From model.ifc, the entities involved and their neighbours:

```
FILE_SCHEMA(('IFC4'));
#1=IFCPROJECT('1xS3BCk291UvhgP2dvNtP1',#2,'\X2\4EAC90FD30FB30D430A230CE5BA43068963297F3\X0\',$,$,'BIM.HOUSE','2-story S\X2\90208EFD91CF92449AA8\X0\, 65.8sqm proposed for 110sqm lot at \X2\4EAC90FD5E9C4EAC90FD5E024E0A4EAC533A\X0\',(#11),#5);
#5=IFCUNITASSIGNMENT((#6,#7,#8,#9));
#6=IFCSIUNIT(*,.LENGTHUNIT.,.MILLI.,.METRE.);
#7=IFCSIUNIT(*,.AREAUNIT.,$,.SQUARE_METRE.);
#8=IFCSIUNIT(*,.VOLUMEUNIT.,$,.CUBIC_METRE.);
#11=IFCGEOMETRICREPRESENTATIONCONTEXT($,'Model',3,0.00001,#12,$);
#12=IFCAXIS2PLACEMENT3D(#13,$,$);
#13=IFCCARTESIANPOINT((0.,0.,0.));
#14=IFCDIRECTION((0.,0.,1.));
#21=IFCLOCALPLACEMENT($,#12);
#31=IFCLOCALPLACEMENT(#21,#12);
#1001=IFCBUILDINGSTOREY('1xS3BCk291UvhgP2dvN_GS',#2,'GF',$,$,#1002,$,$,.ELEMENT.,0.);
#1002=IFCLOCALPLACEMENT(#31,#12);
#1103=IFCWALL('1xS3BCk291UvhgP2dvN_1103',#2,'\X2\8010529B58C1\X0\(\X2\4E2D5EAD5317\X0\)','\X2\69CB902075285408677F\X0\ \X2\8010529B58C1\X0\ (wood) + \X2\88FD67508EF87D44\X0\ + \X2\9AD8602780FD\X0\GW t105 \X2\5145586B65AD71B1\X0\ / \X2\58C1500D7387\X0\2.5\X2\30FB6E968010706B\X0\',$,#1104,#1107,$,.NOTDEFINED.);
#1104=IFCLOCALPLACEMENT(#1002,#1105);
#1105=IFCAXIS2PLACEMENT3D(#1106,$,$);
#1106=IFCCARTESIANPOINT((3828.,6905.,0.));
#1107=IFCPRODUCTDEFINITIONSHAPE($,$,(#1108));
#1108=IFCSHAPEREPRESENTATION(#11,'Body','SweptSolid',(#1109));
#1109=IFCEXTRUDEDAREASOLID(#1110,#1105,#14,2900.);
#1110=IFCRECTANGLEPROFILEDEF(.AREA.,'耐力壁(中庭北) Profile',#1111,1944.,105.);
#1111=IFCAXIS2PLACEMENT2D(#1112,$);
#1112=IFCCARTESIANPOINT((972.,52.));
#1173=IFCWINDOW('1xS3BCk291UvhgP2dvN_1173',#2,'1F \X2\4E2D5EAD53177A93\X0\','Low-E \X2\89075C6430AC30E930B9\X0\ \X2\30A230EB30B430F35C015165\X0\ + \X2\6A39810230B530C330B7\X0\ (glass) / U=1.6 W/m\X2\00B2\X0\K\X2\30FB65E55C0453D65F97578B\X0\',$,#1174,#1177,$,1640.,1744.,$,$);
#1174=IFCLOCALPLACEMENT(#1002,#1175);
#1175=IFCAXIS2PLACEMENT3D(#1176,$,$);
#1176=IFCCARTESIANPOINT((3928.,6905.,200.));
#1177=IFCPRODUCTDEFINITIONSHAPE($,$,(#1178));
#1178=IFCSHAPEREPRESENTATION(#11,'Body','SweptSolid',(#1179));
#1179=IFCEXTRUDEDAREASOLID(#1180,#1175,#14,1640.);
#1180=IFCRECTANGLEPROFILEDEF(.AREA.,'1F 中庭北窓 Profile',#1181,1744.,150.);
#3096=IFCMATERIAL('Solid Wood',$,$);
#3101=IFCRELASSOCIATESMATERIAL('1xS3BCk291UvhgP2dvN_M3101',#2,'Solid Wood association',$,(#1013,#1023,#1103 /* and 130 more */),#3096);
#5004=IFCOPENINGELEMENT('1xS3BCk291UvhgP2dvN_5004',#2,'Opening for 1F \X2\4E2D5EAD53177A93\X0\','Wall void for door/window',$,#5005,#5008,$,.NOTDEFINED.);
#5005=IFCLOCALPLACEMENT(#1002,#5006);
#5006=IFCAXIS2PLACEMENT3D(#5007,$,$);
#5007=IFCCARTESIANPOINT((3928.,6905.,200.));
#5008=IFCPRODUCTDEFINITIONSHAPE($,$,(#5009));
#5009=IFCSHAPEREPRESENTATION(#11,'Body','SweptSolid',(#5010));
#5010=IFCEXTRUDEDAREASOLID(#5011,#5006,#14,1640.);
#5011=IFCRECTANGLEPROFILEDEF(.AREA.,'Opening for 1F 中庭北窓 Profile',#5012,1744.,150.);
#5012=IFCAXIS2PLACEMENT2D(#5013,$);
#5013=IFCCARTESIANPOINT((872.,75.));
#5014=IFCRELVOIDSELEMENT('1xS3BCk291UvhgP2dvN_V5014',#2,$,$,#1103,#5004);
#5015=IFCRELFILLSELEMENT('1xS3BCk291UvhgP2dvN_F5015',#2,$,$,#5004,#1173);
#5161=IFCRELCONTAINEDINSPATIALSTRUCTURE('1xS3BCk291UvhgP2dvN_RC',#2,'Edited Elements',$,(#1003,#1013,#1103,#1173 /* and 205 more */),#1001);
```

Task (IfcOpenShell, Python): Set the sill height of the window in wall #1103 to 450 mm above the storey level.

```python
import numpy as np
import ifcopenshell
import ifcopenshell.api.geometry
import ifcopenshell.geom
import ifcopenshell.util.element
import ifcopenshell.util.placement
import ifcopenshell.util.shape
import ifcopenshell.util.unit

model = ifcopenshell.open("model.ifc")
unit_scale = ifcopenshell.util.unit.calculate_unit_scale(model)

window = model.by_id(1173)
opening = window.FillsVoids[0].RelatingOpeningElement
storey = ifcopenshell.util.element.get_container(window, ifc_class="IfcBuildingStorey")
level = ifcopenshell.util.placement.get_local_placement(storey.ObjectPlacement)[2, 3]

# The opening's origin need not be at the sill, so measure its lowest point.
shape = ifcopenshell.geom.create_shape(ifcopenshell.geom.settings(), opening)
bottom = ifcopenshell.util.shape.get_shape_bottom_elevation(shape, shape.geometry) / unit_scale
dz = level + 0.45 / unit_scale - bottom

shift = np.array([0.0, 0.0, dz])
# The window is not placed relative to its opening, so move both.
for product in (opening, window):
    matrix = ifcopenshell.util.placement.get_local_placement(product.ObjectPlacement)
    matrix[:3, 3] += shift
    ifcopenshell.api.geometry.edit_object_placement(model, product=product, matrix=matrix, is_si=False)

print(f"moved by {dz * unit_scale:+.3f} m")

model.write("model_v2.ifc")
```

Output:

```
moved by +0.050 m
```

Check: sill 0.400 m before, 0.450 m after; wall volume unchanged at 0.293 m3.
